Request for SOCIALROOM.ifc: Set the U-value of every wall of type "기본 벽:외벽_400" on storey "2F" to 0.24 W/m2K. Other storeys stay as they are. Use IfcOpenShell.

First a look at what the model holds.

```python
import ifcopenshell
import ifcopenshell.util.element

model = ifcopenshell.open("SOCIALROOM.ifc")
print(model.schema)
storey = next(s for s in model.by_type("IfcBuildingStorey") if s.Name == "2F")
walls = [e for e in ifcopenshell.util.element.get_decomposition(storey) if e.is_a("IfcWall")]
seen = {}
for e in walls:
    element_type = ifcopenshell.util.element.get_type(e)
    key = (element_type.Name if element_type != e and element_type else None, ifcopenshell.util.element.get_pset(e, "Pset_WallCommon", "ThermalTransmittance"))
    seen[key] = seen.get(key, 0) + 1
for (name, value), count in sorted(seen.items(), key=str):
    print(count, "x", name, "|", value)
```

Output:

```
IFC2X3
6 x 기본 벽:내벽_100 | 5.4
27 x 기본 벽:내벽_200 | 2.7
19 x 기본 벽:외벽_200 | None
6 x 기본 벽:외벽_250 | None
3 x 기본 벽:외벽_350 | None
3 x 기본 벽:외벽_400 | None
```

```python
import ifcopenshell
import ifcopenshell.api.pset
import ifcopenshell.util.element

model = ifcopenshell.open("SOCIALROOM.ifc")

storey = next(s for s in model.by_type("IfcBuildingStorey") if s.Name == "2F")
walls = [e for e in ifcopenshell.util.element.get_decomposition(storey) if e.is_a("IfcWall")]

count = 0
for e in walls:
    element_type = ifcopenshell.util.element.get_type(e)
    if element_type in (None, e) or element_type.Name != "기본 벽:외벽_400":
        continue
    # add_pset returns the element's existing set when there is one.
    pset = ifcopenshell.api.pset.add_pset(model, product=e, name="Pset_WallCommon")
    ifcopenshell.api.pset.edit_pset(model, pset=pset, properties={"ThermalTransmittance": 0.24})
    count += 1

print(count, "walls updated")

model.write("SOCIALROOM_updated.ifc")
```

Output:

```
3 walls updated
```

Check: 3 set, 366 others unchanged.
